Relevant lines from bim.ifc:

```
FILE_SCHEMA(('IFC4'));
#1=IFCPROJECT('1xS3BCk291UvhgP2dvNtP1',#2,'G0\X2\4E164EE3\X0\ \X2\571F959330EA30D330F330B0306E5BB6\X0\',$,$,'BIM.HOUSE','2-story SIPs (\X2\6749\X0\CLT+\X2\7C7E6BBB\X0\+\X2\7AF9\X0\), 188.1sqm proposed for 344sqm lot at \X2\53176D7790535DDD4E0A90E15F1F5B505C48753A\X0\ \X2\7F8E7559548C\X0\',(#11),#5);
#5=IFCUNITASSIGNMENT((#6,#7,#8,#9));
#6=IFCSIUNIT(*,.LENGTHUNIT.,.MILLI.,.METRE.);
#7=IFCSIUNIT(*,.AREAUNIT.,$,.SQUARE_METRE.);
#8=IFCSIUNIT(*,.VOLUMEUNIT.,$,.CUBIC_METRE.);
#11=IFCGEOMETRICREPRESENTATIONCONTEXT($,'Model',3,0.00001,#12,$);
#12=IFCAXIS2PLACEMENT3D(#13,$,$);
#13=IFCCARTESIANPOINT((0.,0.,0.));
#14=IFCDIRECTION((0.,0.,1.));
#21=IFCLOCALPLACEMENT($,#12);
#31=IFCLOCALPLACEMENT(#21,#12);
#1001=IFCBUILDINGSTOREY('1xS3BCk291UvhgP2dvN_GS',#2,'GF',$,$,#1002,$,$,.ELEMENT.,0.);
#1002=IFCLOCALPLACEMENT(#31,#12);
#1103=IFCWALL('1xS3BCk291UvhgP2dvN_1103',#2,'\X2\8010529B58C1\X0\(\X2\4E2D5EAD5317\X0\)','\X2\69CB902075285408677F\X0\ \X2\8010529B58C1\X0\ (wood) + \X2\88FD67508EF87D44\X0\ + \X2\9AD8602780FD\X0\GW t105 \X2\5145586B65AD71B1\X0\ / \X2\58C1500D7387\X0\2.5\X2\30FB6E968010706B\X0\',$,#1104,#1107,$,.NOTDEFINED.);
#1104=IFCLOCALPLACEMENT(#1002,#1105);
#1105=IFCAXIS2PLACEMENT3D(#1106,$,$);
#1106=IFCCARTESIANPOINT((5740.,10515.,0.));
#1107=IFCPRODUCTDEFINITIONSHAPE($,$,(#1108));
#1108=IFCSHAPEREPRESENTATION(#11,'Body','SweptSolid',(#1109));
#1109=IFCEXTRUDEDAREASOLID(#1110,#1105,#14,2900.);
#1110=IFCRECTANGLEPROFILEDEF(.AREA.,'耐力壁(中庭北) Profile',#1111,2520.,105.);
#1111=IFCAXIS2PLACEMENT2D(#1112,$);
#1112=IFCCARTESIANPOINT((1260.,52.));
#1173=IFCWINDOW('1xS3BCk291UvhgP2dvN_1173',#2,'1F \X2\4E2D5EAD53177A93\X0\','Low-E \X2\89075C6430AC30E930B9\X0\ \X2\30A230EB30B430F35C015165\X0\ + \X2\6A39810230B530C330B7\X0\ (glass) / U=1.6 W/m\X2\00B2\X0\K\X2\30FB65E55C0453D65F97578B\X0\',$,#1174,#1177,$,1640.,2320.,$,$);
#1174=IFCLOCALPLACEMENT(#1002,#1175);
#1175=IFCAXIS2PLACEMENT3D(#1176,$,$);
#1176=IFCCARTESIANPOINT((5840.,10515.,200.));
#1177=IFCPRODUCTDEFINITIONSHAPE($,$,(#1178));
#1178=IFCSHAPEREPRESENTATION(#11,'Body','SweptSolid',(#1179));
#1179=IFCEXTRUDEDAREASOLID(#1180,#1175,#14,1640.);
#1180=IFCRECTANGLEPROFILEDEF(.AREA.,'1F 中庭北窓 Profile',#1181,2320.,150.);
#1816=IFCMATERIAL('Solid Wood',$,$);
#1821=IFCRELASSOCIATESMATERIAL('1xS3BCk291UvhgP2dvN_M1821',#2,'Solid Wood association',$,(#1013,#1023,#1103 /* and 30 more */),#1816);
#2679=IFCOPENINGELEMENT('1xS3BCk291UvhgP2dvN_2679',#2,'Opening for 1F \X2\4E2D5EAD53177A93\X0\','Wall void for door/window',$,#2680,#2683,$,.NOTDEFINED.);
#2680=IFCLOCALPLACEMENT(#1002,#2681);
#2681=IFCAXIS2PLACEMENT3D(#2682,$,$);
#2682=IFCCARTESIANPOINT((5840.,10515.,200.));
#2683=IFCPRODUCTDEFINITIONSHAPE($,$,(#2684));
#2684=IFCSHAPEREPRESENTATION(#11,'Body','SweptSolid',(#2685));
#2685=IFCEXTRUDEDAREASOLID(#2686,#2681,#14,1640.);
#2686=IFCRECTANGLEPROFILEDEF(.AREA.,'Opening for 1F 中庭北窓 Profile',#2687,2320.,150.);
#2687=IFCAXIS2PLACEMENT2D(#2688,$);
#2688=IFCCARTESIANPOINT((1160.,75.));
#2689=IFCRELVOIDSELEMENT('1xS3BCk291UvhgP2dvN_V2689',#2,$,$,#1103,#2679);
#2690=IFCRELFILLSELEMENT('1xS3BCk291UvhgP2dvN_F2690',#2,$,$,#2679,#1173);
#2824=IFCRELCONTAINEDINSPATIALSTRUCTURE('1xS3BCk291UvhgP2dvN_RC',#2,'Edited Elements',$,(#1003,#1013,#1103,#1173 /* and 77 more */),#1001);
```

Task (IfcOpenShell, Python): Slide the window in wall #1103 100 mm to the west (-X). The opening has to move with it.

```python
import ifcopenshell
import ifcopenshell.api.geometry
import ifcopenshell.util.placement

model = ifcopenshell.open("bim.ifc")

window = model.by_guid("1xS3BCk291UvhgP2dvN_1173")
opening = window.FillsVoids[0].RelatingOpeningElement
wall = opening.VoidsElements[0].RelatingBuildingElement

wall_matrix = ifcopenshell.util.placement.get_local_placement(wall.ObjectPlacement)
shift = wall_matrix[:3, 0] * -100.0
before = ifcopenshell.util.placement.get_local_placement(window.ObjectPlacement)[:3, 3].copy()

# The window is not placed relative to its opening, so move both.
for product in (opening, window):
    matrix = ifcopenshell.util.placement.get_local_placement(product.ObjectPlacement)
    matrix[:3, 3] += shift
    ifcopenshell.api.geometry.edit_object_placement(model, product=product, matrix=matrix, is_si=False)

after = ifcopenshell.util.placement.get_local_placement(window.ObjectPlacement)[:3, 3]
print("window moved by", (after - before).round(3) + 0.0)

model.write("bim_updated.ifc")
```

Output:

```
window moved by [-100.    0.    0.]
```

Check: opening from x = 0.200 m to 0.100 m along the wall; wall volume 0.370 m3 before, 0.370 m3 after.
